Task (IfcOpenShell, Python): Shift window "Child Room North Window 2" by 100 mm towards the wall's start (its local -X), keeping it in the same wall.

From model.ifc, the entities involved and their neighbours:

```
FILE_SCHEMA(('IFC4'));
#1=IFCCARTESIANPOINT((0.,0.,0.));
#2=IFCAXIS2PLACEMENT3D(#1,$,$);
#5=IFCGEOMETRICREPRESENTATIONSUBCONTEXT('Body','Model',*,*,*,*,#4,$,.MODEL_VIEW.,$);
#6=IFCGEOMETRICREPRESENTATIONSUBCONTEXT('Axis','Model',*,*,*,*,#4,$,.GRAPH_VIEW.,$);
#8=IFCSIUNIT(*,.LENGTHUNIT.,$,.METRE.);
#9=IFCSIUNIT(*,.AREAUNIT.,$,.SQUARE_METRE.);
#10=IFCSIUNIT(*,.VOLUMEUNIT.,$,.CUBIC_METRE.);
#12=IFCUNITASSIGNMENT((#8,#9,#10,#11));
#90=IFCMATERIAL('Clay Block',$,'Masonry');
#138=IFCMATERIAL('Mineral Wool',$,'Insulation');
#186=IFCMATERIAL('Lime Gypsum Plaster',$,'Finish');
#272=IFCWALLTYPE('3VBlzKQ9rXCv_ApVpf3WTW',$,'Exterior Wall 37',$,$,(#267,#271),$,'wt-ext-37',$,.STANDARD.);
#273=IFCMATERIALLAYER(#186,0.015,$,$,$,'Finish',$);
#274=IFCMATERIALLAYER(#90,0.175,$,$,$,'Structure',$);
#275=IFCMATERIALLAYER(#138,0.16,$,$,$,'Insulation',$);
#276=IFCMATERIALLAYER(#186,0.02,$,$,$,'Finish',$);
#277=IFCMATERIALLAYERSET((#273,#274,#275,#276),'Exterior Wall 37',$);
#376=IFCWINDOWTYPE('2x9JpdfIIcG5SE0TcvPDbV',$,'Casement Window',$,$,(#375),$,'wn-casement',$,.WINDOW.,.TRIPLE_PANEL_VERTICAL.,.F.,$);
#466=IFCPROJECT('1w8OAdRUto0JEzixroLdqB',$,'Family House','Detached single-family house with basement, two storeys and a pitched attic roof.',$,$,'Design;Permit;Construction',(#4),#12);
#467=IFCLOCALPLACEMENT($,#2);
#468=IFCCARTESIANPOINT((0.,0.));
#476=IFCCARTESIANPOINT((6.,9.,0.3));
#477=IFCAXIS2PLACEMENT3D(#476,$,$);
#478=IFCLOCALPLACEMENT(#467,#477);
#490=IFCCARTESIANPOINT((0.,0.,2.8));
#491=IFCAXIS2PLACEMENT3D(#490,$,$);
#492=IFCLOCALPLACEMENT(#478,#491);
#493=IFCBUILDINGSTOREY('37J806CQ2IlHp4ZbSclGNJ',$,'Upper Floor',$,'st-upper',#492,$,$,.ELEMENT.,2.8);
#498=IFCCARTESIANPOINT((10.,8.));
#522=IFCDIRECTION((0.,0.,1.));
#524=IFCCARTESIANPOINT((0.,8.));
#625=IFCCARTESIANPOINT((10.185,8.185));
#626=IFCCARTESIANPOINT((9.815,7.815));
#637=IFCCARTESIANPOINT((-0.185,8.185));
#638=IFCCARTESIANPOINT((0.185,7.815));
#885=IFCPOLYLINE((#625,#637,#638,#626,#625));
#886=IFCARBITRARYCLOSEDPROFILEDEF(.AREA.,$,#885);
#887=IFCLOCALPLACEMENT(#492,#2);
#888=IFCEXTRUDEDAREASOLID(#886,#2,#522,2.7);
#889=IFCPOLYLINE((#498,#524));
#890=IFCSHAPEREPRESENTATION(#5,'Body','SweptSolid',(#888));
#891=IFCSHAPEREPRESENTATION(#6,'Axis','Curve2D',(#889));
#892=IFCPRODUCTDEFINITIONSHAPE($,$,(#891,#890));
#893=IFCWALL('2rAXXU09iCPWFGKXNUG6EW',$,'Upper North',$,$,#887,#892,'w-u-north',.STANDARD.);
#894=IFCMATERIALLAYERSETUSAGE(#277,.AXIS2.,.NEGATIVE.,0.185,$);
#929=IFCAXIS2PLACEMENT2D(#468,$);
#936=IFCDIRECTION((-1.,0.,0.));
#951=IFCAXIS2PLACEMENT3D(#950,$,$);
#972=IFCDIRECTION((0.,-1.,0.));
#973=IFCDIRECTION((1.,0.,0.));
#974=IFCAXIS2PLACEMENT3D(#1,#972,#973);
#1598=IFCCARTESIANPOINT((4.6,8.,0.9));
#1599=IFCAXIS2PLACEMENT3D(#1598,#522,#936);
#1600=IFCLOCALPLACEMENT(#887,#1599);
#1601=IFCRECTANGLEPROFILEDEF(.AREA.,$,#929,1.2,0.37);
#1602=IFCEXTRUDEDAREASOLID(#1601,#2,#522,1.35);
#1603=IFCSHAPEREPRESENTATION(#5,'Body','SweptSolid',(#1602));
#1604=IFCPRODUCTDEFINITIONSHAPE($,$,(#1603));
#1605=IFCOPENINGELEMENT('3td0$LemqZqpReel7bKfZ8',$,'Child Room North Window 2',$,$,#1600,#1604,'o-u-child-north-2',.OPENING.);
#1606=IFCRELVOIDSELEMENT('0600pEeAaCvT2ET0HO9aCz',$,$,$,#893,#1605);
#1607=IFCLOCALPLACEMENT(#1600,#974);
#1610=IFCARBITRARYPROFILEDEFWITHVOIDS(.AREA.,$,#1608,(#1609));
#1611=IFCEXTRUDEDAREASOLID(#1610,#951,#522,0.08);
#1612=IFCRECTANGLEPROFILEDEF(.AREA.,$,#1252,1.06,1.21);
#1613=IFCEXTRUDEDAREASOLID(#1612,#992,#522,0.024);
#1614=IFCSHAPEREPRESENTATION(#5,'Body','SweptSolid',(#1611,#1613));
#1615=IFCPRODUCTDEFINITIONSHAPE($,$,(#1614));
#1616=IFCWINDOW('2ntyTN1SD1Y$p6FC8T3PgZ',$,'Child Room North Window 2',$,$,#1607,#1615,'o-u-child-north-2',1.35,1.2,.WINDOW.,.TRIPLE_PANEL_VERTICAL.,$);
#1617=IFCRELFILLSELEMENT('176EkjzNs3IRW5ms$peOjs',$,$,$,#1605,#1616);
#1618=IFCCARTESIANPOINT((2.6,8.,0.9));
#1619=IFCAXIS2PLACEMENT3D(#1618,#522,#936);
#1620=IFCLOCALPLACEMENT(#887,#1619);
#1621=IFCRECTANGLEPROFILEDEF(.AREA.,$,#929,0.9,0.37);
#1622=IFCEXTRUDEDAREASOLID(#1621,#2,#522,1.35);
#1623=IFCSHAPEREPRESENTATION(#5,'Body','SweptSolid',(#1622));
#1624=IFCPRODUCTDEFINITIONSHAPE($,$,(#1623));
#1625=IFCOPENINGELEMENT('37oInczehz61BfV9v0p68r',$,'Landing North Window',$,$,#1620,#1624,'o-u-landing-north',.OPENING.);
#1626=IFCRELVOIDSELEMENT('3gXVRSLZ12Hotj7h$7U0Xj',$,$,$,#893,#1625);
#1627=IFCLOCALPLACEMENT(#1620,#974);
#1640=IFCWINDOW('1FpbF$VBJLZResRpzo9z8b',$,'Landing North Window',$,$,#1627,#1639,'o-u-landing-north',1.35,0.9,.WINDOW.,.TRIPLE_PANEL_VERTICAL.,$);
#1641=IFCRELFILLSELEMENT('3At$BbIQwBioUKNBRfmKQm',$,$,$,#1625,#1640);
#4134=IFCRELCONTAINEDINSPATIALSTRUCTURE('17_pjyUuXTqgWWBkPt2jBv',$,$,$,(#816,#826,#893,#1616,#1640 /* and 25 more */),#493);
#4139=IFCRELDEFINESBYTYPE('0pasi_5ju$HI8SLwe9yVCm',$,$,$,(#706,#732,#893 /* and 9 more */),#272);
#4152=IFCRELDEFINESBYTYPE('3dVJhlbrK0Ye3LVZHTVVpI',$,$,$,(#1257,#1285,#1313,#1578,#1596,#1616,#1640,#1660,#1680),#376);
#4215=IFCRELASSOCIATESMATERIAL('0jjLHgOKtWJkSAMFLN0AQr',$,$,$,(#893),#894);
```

```python
import ifcopenshell
import ifcopenshell.api.geometry
import ifcopenshell.util.placement

model = ifcopenshell.open("model.ifc")

window = model.by_guid("2ntyTN1SD1Y$p6FC8T3PgZ")
opening = window.FillsVoids[0].RelatingOpeningElement
wall = opening.VoidsElements[0].RelatingBuildingElement

wall_matrix = ifcopenshell.util.placement.get_local_placement(wall.ObjectPlacement)
shift = wall_matrix[:3, 0] * -0.1
before = ifcopenshell.util.placement.get_local_placement(window.ObjectPlacement)[:3, 3].copy()

# The window is placed relative to its opening, so it follows when the opening moves.
matrix = ifcopenshell.util.placement.get_local_placement(opening.ObjectPlacement)
matrix[:3, 3] += shift
ifcopenshell.api.geometry.edit_object_placement(
    model, product=opening, matrix=matrix, is_si=False, should_transform_children=True
)

after = ifcopenshell.util.placement.get_local_placement(window.ObjectPlacement)[:3, 3]
print("window moved by", (after - before).round(3) + 0.0)

model.write("model-out.ifc")
```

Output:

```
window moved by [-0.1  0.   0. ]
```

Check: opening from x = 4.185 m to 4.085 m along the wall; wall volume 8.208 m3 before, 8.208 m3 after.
